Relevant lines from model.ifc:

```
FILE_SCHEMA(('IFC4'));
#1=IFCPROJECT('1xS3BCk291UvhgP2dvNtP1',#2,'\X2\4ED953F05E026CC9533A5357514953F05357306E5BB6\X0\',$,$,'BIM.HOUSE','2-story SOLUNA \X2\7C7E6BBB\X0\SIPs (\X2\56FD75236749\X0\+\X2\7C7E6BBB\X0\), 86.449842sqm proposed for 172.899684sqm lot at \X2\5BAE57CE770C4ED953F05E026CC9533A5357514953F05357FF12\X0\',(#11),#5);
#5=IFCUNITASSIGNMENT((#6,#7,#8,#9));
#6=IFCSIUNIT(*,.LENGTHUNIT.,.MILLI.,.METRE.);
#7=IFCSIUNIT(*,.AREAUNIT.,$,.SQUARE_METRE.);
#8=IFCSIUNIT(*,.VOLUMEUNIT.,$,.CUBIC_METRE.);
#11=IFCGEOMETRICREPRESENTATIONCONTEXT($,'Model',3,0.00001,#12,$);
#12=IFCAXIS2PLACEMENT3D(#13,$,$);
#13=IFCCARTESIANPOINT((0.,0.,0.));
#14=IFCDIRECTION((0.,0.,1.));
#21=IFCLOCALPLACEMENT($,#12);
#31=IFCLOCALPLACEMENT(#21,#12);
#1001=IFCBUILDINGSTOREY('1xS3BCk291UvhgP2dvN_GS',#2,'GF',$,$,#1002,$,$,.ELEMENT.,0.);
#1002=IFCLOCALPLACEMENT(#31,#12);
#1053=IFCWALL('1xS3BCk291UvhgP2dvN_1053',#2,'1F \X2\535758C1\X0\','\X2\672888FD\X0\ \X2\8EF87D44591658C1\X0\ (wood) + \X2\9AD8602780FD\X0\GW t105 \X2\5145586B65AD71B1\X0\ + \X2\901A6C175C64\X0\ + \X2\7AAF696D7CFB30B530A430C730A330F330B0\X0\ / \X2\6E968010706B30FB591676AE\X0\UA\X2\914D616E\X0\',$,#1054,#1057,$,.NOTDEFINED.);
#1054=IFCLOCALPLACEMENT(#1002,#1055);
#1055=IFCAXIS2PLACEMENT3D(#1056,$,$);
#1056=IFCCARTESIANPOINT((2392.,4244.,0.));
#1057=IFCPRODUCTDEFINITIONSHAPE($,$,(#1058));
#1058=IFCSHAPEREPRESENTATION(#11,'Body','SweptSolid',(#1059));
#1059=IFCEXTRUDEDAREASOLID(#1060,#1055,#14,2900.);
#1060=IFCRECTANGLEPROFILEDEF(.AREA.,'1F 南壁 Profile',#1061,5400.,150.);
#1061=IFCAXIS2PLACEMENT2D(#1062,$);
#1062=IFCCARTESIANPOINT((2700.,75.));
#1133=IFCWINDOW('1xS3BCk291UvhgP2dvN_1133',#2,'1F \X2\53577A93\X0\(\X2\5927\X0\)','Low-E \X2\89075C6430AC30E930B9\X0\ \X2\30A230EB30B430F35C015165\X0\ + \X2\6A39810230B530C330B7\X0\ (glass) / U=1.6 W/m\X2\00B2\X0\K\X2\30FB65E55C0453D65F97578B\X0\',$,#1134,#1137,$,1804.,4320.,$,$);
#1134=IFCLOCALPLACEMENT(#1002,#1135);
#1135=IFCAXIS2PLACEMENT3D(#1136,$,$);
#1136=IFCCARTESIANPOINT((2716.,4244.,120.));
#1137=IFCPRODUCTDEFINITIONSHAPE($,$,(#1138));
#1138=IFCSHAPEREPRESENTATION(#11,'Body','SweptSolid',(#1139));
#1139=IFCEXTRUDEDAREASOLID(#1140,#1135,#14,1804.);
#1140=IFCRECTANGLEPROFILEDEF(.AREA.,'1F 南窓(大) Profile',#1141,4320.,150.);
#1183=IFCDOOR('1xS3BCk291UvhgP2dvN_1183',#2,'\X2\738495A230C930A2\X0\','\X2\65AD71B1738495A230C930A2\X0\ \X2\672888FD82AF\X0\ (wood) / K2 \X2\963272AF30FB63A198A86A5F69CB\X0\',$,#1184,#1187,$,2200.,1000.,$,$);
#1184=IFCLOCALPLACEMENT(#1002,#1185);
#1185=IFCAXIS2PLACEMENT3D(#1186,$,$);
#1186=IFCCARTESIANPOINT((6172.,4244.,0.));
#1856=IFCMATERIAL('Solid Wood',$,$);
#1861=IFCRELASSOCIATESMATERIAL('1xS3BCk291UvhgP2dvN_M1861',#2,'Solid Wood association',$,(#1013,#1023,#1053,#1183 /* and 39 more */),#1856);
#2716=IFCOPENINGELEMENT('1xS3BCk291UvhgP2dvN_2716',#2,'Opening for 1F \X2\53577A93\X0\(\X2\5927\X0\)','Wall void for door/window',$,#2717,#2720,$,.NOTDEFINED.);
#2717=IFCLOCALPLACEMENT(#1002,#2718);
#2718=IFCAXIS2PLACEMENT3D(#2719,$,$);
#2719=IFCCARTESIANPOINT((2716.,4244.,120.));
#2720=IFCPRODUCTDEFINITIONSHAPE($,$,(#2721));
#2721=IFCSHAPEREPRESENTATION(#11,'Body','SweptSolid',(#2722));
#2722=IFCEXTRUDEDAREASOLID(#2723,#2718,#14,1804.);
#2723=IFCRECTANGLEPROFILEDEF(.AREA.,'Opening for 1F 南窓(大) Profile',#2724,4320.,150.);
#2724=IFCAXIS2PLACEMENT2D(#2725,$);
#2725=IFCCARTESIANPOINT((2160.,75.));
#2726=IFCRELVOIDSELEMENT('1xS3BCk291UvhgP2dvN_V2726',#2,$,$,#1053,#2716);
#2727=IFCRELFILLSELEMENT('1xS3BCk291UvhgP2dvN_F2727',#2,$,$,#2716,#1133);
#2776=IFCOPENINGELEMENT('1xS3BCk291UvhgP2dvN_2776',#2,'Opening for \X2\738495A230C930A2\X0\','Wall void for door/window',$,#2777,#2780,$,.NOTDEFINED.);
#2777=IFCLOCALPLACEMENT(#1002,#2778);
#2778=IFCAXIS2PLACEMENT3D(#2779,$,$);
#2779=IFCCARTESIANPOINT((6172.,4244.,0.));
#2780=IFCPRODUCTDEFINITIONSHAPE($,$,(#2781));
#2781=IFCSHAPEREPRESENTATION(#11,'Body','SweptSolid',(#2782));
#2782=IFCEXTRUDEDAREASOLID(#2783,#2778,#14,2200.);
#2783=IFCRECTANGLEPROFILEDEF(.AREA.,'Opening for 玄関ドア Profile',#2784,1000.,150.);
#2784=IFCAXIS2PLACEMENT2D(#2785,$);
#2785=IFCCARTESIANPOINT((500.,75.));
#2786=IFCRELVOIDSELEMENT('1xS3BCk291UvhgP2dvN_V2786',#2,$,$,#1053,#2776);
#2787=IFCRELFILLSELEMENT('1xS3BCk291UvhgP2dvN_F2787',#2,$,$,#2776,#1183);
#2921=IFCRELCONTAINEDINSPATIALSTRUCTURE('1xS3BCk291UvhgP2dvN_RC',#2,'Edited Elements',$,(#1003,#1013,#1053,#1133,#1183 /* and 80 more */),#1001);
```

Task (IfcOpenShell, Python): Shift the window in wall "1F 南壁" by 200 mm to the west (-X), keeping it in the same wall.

```python
import ifcopenshell
import ifcopenshell.api.geometry
import ifcopenshell.util.placement

model = ifcopenshell.open("model.ifc")

window = model.by_id(1133)
opening = window.FillsVoids[0].RelatingOpeningElement
wall = opening.VoidsElements[0].RelatingBuildingElement

wall_matrix = ifcopenshell.util.placement.get_local_placement(wall.ObjectPlacement)
shift = wall_matrix[:3, 0] * -200.0
before = ifcopenshell.util.placement.get_local_placement(window.ObjectPlacement)[:3, 3].copy()

# The window is not placed relative to its opening, so move both.
for product in (opening, window):
    matrix = ifcopenshell.util.placement.get_local_placement(product.ObjectPlacement)
    matrix[:3, 3] += shift
    ifcopenshell.api.geometry.edit_object_placement(model, product=product, matrix=matrix, is_si=False)

after = ifcopenshell.util.placement.get_local_placement(window.ObjectPlacement)[:3, 3]
print("window moved by", (after - before).round(3) + 0.0)

model.write("model_edited.ifc")
```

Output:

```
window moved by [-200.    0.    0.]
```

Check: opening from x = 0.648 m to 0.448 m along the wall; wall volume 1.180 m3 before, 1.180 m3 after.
